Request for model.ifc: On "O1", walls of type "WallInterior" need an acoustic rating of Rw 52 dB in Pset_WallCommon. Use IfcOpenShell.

First a look at what the model holds.

```python
import ifcopenshell
import ifcopenshell.util.element

model = ifcopenshell.open("model.ifc")
print(model.schema)
storey = next(s for s in model.by_type("IfcBuildingStorey") if s.Name == "O1")
walls = [e for e in ifcopenshell.util.element.get_decomposition(storey) if e.is_a("IfcWall")]
seen = {}
for e in walls:
    element_type = ifcopenshell.util.element.get_type(e)
    key = (element_type.Name if element_type != e and element_type else None, ifcopenshell.util.element.get_pset(e, "Pset_WallCommon", "AcousticRating"))
    seen[key] = seen.get(key, 0) + 1
for (name, value), count in sorted(seen.items(), key=str):
    print(count, "x", name, "|", value)
```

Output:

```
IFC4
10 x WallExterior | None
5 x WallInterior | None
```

```python
import ifcopenshell
import ifcopenshell.api.pset
import ifcopenshell.util.element

model = ifcopenshell.open("model.ifc")

storey = next(s for s in model.by_type("IfcBuildingStorey") if s.Name == "O1")
walls = [e for e in ifcopenshell.util.element.get_decomposition(storey) if e.is_a("IfcWall")]

count = 0
for e in walls:
    element_type = ifcopenshell.util.element.get_type(e)
    if element_type in (None, e) or element_type.Name != "WallInterior":
        continue
    # add_pset returns the element's existing set when there is one.
    pset = ifcopenshell.api.pset.add_pset(model, product=e, name="Pset_WallCommon")
    ifcopenshell.api.pset.edit_pset(model, pset=pset, properties={"AcousticRating": "Rw 52 dB"})
    count += 1

print(count, "walls updated")

model.write("model_updated.ifc")
```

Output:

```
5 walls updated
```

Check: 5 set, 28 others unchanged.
